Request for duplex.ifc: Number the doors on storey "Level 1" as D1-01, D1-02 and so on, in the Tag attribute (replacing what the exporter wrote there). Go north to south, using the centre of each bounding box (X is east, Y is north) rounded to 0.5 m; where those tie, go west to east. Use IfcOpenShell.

First a look at what the model holds.

```python
import ifcopenshell
import ifcopenshell.util.element
import ifcopenshell.util.placement

model = ifcopenshell.open("duplex.ifc")
print(model.schema)
storey = next(s for s in model.by_type("IfcBuildingStorey") if s.Name == "Level 1")
doors = [e for e in ifcopenshell.util.element.get_decomposition(storey) if e.is_a("IfcDoor")]
for e in sorted(doors, key=lambda e: e.id()):
    origin = ifcopenshell.util.placement.get_local_placement(e.ObjectPlacement)[:3, 3]
    print(e.id(), e.Tag, e.Name, origin.round(2) + 0.0, sep=" | ")
```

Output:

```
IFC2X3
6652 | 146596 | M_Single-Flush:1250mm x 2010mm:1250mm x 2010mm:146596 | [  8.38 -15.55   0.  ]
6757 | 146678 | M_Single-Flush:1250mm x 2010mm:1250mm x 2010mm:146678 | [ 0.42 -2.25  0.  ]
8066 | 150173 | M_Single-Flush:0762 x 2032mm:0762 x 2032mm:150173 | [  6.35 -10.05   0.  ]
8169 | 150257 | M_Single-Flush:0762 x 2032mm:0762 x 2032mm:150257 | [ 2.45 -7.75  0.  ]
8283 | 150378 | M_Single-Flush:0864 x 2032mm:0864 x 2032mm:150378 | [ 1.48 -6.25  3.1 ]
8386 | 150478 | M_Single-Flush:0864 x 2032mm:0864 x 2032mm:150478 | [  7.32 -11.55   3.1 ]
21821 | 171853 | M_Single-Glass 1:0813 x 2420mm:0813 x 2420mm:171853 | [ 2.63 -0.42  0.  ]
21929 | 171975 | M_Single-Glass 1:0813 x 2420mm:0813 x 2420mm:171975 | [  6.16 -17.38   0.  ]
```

```python
import ifcopenshell
import ifcopenshell.geom
import ifcopenshell.util.element
import ifcopenshell.util.shape

model = ifcopenshell.open("duplex.ifc")
settings = ifcopenshell.geom.settings()
settings.set("use-world-coords", True)


def centre(element):
    shape = ifcopenshell.geom.create_shape(settings, element)
    return ifcopenshell.util.shape.get_bbox_centroid(shape.geometry)


storey = next(s for s in model.by_type("IfcBuildingStorey") if s.Name == "Level 1")
doors = [e for e in ifcopenshell.util.element.get_decomposition(storey) if e.is_a("IfcDoor")]

# Insertion points can sit at a corner or the storey origin, so sort by the geometry (in metres).
centres = {e: centre(e) for e in doors}
doors.sort(key=lambda e: (-round(centres[e][1] / 0.5), centres[e][0]))

for i, e in enumerate(doors, start=1):
    number = f"D1-{i:02d}"
    e.Tag = number
    print(e.id(), number)

model.write("duplex_v2.ifc")
```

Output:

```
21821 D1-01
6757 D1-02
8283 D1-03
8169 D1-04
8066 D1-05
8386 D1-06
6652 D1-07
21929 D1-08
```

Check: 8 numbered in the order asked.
